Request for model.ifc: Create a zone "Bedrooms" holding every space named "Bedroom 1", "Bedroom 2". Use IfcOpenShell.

First a look at what the model holds.

```python
import ifcopenshell

model = ifcopenshell.open("model.ifc")
print(model.schema)
seen = {}
for space in model.by_type("IfcSpace"):
    seen[space.LongName] = seen.get(space.LongName, 0) + 1
for name, count in sorted(seen.items(), key=str):
    print(count, "x", name)
print("zones:", [z.Name for z in model.by_type("IfcZone")][:20])
```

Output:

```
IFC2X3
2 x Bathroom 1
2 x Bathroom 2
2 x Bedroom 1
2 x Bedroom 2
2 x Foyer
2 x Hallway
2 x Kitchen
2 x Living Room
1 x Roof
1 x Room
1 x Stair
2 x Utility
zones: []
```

```python
import ifcopenshell
import ifcopenshell.api.group
import ifcopenshell.api.root

model = ifcopenshell.open("model.ifc")

names = {"Bedroom 1", "Bedroom 2"}
spaces = [s for s in model.by_type("IfcSpace") if s.LongName in names]

zone = ifcopenshell.api.root.create_entity(model, ifc_class="IfcZone", name="Bedrooms")
ifcopenshell.api.group.assign_group(model, products=spaces, group=zone)
print(len(spaces), "spaces in", zone.Name)

model.write("model_rev.ifc")
```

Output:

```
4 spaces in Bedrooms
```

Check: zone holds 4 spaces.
